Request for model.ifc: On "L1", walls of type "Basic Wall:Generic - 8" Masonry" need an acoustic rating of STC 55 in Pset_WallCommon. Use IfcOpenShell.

First a look at what the model holds.

```python
import ifcopenshell
import ifcopenshell.util.element

model = ifcopenshell.open("model.ifc")
print(model.schema)
storey = next(s for s in model.by_type("IfcBuildingStorey") if s.Name == "L1")
walls = [e for e in ifcopenshell.util.element.get_decomposition(storey) if e.is_a("IfcWall")]
seen = {}
for e in walls:
    element_type = ifcopenshell.util.element.get_type(e)
    key = (element_type.Name if element_type != e and element_type else None, ifcopenshell.util.element.get_pset(e, "Pset_WallCommon", "AcousticRating"))
    seen[key] = seen.get(key, 0) + 1
for (name, value), count in sorted(seen.items(), key=str):
    print(count, "x", name, "|", value)
```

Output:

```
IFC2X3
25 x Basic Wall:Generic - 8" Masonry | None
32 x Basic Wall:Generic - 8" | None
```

```python
import ifcopenshell
import ifcopenshell.api.pset
import ifcopenshell.util.element

model = ifcopenshell.open("model.ifc")

storey = next(s for s in model.by_type("IfcBuildingStorey") if s.Name == "L1")
walls = [e for e in ifcopenshell.util.element.get_decomposition(storey) if e.is_a("IfcWall")]

count = 0
for e in walls:
    element_type = ifcopenshell.util.element.get_type(e)
    if element_type in (None, e) or element_type.Name != 'Basic Wall:Generic - 8" Masonry':
        continue
    # add_pset returns the element's existing set when there is one.
    pset = ifcopenshell.api.pset.add_pset(model, product=e, name="Pset_WallCommon")
    ifcopenshell.api.pset.edit_pset(model, pset=pset, properties={"AcousticRating": "STC 55"})
    count += 1

print(count, "walls updated")

model.write("model_v2.ifc")
```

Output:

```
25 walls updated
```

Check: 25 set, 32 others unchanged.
